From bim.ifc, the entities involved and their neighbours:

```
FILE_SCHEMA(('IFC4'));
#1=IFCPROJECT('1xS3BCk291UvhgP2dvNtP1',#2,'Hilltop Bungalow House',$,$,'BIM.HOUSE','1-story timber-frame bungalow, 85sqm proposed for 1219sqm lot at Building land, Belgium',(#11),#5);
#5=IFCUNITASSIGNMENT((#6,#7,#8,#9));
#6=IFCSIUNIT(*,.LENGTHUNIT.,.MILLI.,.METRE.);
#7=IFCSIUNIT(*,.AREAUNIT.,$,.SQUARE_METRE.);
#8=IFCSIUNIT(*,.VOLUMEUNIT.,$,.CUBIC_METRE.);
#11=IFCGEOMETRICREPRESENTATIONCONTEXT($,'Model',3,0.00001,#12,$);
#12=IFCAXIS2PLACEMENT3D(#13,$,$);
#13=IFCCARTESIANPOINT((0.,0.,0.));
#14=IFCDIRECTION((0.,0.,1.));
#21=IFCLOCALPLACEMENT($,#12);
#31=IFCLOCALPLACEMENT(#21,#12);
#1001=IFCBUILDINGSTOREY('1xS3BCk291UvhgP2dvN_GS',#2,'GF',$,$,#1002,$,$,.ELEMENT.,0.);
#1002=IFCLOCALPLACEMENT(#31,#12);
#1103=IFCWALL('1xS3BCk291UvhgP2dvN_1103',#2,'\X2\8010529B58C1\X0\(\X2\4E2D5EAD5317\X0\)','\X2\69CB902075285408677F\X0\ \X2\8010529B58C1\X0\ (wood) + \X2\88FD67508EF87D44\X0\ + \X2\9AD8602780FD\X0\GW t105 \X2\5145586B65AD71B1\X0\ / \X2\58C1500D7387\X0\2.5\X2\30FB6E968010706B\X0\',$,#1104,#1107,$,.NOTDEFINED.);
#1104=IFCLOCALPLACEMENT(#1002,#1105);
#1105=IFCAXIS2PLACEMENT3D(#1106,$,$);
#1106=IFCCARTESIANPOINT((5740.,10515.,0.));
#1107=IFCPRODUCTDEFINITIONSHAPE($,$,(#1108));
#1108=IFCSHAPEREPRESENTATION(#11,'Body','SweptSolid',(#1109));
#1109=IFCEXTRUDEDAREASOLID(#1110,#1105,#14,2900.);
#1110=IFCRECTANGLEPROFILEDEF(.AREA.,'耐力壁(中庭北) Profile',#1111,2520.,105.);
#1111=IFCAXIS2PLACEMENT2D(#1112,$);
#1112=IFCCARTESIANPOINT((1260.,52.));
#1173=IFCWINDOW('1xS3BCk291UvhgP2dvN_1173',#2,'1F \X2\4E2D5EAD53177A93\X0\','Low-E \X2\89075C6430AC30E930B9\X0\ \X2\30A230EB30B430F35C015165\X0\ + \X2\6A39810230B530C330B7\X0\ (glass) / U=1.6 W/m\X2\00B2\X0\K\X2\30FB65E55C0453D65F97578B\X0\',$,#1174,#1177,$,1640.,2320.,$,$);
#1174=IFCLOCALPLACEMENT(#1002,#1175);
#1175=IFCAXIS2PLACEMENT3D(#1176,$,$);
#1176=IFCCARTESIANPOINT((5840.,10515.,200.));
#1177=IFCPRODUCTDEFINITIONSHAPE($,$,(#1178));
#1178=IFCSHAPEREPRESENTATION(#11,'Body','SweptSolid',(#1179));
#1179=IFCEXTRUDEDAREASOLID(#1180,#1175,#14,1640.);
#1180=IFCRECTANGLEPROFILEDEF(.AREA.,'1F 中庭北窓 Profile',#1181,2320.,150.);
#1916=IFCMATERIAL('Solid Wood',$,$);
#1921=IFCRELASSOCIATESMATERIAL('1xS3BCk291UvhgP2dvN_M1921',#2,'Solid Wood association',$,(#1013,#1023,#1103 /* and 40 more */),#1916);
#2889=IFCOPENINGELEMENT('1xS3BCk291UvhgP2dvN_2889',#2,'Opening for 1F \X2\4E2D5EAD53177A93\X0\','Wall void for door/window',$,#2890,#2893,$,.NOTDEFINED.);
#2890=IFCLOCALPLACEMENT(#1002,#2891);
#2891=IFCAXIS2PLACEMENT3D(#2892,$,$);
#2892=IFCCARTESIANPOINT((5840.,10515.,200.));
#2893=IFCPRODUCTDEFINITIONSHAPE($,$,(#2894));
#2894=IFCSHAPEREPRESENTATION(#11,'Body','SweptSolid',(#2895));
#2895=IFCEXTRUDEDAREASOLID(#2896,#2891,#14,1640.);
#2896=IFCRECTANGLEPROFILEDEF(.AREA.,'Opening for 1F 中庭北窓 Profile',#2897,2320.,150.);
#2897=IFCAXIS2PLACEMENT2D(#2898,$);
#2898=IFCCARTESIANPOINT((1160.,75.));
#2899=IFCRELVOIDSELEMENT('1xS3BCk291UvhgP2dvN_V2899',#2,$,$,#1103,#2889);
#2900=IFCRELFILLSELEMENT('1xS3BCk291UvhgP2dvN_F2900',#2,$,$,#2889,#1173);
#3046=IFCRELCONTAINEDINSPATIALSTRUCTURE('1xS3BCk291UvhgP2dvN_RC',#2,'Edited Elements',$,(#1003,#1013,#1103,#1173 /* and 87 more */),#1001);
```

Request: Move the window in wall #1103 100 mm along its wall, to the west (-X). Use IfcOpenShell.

```python
import ifcopenshell
import ifcopenshell.api.geometry
import ifcopenshell.util.placement
import ifcopenshell.util.unit

model = ifcopenshell.open("bim.ifc")
unit_scale = ifcopenshell.util.unit.calculate_unit_scale(model)

window = model.by_id(1173)
opening = window.FillsVoids[0].RelatingOpeningElement
wall = opening.VoidsElements[0].RelatingBuildingElement

wall_matrix = ifcopenshell.util.placement.get_local_placement(wall.ObjectPlacement)
shift = wall_matrix[:3, 0] * -0.1 / unit_scale
before = ifcopenshell.util.placement.get_local_placement(window.ObjectPlacement)[:3, 3].copy()

# The window is not placed relative to its opening, so move both.
for product in (opening, window):
    matrix = ifcopenshell.util.placement.get_local_placement(product.ObjectPlacement)
    matrix[:3, 3] += shift
    ifcopenshell.api.geometry.edit_object_placement(model, product=product, matrix=matrix, is_si=False)

after = ifcopenshell.util.placement.get_local_placement(window.ObjectPlacement)[:3, 3]
print("window moved by", (after - before).round(3) + 0.0)

model.write("bim-out.ifc")
```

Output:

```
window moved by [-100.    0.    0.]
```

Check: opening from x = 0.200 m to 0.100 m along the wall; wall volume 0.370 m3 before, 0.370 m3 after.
